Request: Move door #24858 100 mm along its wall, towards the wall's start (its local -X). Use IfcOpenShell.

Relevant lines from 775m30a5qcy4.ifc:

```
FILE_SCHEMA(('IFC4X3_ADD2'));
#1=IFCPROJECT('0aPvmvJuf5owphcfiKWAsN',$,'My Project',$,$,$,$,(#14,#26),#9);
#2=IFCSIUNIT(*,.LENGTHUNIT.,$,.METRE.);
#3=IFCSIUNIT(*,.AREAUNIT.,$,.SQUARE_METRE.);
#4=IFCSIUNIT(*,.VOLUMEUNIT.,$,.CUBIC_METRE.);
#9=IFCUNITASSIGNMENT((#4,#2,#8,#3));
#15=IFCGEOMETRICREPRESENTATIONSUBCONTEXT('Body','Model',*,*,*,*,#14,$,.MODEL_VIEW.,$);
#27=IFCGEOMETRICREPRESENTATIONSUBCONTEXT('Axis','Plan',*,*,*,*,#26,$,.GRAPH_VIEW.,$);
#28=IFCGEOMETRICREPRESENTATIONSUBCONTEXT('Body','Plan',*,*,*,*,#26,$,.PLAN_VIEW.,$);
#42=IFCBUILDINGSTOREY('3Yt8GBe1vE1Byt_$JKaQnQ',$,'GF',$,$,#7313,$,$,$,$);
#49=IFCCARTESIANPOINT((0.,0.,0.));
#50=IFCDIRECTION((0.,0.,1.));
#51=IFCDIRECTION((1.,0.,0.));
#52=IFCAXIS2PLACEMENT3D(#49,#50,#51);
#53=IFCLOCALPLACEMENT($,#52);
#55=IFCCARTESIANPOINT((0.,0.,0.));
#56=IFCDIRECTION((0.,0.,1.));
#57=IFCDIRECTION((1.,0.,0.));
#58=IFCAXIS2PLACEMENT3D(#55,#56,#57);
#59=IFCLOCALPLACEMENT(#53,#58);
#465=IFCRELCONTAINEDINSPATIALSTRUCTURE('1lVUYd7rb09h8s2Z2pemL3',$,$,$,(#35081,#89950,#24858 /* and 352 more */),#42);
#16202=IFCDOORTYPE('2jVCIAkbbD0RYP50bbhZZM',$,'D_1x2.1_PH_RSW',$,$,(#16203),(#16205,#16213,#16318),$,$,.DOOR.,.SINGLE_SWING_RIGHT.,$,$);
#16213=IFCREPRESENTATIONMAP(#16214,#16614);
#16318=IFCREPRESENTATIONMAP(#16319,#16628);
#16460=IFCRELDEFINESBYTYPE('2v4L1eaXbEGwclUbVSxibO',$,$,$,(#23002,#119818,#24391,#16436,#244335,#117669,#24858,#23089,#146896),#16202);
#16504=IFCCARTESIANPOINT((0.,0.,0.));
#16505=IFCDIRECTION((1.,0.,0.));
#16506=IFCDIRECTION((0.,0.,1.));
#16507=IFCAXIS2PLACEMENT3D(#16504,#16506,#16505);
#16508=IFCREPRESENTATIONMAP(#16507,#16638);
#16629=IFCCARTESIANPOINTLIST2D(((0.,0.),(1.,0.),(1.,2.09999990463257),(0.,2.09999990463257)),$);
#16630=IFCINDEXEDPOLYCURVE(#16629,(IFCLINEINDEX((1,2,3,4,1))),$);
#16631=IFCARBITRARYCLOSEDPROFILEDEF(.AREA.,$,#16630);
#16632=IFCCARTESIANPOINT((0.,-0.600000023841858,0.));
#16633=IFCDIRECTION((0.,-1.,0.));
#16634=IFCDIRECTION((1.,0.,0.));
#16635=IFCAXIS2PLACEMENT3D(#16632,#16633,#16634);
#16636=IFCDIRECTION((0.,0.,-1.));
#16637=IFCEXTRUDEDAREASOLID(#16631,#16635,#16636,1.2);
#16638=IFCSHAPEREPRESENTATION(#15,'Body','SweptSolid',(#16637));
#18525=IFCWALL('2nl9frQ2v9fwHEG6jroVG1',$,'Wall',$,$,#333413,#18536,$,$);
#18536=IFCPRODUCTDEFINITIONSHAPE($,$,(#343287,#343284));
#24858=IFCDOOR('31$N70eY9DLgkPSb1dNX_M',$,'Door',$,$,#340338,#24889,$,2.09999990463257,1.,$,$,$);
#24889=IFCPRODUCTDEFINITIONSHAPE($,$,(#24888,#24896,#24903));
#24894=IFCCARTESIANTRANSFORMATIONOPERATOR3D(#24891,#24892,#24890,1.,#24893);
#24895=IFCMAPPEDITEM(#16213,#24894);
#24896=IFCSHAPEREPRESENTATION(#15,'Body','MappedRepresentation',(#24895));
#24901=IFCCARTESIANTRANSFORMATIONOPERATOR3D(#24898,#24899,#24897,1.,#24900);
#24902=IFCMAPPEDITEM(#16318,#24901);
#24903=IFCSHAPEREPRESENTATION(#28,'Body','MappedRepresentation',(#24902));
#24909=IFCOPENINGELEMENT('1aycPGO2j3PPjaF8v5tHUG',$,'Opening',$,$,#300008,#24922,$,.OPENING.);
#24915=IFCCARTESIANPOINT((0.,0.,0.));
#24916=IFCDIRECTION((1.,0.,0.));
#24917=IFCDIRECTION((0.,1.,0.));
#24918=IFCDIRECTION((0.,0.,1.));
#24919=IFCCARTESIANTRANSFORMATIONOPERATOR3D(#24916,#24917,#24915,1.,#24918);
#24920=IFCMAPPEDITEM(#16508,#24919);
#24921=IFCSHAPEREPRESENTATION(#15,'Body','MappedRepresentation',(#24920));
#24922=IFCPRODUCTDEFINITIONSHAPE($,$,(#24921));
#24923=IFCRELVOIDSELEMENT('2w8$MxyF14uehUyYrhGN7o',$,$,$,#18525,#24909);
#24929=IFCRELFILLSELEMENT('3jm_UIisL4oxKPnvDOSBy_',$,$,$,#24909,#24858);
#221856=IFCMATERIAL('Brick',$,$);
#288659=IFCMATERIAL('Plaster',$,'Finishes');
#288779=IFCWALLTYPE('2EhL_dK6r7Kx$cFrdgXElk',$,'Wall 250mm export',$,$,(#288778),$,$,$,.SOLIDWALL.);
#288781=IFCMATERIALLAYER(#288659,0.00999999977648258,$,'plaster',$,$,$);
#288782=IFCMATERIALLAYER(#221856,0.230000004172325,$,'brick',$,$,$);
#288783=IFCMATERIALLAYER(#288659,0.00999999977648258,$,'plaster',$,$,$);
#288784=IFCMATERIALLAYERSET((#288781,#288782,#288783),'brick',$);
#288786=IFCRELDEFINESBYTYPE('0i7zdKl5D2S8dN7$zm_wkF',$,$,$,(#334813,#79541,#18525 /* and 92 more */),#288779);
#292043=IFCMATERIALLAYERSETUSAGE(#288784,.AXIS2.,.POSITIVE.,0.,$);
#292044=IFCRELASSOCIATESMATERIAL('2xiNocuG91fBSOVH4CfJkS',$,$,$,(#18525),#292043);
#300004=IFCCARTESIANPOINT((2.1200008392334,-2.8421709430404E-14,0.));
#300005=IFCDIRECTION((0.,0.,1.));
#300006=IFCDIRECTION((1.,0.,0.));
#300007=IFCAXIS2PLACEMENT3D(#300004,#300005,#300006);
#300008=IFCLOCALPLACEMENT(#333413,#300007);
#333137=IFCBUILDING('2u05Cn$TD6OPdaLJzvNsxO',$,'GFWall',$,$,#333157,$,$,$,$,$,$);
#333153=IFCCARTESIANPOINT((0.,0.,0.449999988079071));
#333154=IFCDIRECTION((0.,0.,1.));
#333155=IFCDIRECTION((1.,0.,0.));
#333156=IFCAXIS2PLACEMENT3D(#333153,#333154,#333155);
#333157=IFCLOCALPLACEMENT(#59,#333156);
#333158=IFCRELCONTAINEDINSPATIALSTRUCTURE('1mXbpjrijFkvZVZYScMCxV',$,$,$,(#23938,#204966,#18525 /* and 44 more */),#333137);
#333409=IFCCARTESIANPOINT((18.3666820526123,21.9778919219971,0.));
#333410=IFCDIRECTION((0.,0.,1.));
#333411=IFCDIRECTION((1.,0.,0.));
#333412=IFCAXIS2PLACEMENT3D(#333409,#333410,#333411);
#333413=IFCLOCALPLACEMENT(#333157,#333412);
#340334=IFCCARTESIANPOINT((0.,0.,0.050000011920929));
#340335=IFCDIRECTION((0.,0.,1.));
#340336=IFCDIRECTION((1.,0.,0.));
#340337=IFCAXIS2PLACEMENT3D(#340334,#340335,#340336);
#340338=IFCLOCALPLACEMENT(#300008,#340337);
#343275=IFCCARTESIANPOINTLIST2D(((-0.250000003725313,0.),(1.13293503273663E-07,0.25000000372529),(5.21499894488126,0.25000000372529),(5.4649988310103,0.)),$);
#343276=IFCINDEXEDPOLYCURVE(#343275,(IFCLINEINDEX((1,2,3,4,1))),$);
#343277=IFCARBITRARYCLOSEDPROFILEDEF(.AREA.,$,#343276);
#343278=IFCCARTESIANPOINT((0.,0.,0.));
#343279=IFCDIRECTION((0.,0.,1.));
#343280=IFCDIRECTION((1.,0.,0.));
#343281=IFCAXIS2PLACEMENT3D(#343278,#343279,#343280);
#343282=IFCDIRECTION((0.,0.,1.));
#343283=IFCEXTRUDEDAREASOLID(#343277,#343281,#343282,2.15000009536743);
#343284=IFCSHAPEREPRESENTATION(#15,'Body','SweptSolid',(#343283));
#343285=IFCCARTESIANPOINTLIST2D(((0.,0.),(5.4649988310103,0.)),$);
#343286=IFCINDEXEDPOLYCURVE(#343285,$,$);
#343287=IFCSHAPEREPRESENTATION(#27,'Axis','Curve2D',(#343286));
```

```python
import ifcopenshell
import ifcopenshell.api.geometry
import ifcopenshell.util.placement

model = ifcopenshell.open("775m30a5qcy4.ifc")

door = model.by_guid("31$N70eY9DLgkPSb1dNX_M")
opening = door.FillsVoids[0].RelatingOpeningElement
wall = opening.VoidsElements[0].RelatingBuildingElement

wall_matrix = ifcopenshell.util.placement.get_local_placement(wall.ObjectPlacement)
shift = wall_matrix[:3, 0] * -0.1
before = ifcopenshell.util.placement.get_local_placement(door.ObjectPlacement)[:3, 3].copy()

# The door is placed relative to its opening, so it follows when the opening moves.
matrix = ifcopenshell.util.placement.get_local_placement(opening.ObjectPlacement)
matrix[:3, 3] += shift
ifcopenshell.api.geometry.edit_object_placement(
    model, product=opening, matrix=matrix, is_si=False, should_transform_children=True
)

after = ifcopenshell.util.placement.get_local_placement(door.ObjectPlacement)[:3, 3]
print("door moved by", (after - before).round(3) + 0.0)

model.write("775m30a5qcy4_v2.ifc")
```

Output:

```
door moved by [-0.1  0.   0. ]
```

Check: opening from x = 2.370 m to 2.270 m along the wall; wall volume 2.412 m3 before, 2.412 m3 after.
